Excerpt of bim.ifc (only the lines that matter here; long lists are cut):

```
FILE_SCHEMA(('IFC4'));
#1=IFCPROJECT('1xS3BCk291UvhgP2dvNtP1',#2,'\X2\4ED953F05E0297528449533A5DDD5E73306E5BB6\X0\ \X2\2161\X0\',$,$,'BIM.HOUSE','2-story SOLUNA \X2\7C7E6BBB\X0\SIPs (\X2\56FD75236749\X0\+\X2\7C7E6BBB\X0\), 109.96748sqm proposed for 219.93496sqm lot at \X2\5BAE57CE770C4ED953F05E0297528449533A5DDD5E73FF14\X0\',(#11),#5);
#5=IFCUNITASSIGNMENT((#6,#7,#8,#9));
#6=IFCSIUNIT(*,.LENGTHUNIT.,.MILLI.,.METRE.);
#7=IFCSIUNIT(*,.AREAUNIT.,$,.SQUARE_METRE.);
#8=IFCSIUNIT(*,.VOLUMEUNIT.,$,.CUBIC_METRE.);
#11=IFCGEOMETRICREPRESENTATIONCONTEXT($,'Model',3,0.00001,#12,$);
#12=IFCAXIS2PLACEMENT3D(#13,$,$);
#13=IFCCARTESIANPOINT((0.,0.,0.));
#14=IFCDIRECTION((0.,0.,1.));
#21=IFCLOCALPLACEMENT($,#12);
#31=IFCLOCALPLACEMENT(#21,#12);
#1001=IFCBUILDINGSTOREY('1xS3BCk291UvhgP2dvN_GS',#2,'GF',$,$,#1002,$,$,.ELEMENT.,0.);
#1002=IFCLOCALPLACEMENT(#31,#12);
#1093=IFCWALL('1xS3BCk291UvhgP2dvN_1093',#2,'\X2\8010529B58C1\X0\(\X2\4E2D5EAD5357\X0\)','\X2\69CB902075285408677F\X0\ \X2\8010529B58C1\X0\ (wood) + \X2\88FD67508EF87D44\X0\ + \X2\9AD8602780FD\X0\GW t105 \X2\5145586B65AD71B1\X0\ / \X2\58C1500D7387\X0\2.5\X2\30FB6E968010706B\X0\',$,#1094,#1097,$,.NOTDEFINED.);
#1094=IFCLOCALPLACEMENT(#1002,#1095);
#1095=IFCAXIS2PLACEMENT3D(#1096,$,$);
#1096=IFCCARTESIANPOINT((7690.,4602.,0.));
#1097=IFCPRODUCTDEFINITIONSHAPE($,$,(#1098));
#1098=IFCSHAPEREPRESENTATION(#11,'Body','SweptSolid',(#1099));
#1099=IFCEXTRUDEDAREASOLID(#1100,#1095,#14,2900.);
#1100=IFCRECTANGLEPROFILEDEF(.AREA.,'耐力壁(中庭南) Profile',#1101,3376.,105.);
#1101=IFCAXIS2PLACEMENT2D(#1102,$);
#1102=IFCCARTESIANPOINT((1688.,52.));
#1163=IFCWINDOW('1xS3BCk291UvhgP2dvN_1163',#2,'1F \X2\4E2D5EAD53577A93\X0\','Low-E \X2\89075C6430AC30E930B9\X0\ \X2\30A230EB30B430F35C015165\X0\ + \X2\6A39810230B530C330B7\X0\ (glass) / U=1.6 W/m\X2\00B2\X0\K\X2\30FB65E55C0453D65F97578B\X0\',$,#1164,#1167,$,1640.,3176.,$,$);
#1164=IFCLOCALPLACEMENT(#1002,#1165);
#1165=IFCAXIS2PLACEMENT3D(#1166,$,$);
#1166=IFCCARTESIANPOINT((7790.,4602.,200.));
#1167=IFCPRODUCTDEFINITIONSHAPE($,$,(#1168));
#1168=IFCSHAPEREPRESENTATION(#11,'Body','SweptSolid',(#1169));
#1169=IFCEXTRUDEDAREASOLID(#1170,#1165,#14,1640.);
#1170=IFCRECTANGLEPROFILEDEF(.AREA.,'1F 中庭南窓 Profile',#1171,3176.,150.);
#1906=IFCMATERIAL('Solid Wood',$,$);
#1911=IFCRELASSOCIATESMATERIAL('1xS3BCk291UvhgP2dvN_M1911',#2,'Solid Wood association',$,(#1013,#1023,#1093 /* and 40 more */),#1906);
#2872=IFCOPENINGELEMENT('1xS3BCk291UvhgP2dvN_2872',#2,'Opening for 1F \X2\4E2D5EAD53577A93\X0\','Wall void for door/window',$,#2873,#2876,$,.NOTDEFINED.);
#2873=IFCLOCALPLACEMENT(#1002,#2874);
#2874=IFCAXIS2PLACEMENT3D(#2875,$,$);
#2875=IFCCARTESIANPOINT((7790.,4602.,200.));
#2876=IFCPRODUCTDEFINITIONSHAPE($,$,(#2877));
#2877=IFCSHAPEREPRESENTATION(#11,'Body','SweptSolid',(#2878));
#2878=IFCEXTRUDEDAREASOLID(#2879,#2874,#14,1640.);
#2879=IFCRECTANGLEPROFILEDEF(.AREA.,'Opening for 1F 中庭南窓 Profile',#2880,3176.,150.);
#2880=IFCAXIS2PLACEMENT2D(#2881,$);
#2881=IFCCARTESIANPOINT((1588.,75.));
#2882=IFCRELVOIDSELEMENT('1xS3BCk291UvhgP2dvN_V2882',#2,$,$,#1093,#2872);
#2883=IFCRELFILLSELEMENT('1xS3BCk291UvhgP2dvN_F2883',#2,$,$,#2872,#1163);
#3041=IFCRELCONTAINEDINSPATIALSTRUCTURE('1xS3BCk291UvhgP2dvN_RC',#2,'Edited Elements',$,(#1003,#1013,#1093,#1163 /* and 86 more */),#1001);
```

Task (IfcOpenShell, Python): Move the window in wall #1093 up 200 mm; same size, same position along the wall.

```python
import numpy as np
import ifcopenshell
import ifcopenshell.api.geometry
import ifcopenshell.util.placement
import ifcopenshell.util.unit

model = ifcopenshell.open("bim.ifc")
unit_scale = ifcopenshell.util.unit.calculate_unit_scale(model)

window = model.by_guid("1xS3BCk291UvhgP2dvN_1163")
opening = window.FillsVoids[0].RelatingOpeningElement
dz = 200.0

shift = np.array([0.0, 0.0, dz])
# The window is not placed relative to its opening, so move both.
for product in (opening, window):
    matrix = ifcopenshell.util.placement.get_local_placement(product.ObjectPlacement)
    matrix[:3, 3] += shift
    ifcopenshell.api.geometry.edit_object_placement(model, product=product, matrix=matrix, is_si=False)

print(f"moved by {dz * unit_scale:+.3f} m")

model.write("bim_v2.ifc")
```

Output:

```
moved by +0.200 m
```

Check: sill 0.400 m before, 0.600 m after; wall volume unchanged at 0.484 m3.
